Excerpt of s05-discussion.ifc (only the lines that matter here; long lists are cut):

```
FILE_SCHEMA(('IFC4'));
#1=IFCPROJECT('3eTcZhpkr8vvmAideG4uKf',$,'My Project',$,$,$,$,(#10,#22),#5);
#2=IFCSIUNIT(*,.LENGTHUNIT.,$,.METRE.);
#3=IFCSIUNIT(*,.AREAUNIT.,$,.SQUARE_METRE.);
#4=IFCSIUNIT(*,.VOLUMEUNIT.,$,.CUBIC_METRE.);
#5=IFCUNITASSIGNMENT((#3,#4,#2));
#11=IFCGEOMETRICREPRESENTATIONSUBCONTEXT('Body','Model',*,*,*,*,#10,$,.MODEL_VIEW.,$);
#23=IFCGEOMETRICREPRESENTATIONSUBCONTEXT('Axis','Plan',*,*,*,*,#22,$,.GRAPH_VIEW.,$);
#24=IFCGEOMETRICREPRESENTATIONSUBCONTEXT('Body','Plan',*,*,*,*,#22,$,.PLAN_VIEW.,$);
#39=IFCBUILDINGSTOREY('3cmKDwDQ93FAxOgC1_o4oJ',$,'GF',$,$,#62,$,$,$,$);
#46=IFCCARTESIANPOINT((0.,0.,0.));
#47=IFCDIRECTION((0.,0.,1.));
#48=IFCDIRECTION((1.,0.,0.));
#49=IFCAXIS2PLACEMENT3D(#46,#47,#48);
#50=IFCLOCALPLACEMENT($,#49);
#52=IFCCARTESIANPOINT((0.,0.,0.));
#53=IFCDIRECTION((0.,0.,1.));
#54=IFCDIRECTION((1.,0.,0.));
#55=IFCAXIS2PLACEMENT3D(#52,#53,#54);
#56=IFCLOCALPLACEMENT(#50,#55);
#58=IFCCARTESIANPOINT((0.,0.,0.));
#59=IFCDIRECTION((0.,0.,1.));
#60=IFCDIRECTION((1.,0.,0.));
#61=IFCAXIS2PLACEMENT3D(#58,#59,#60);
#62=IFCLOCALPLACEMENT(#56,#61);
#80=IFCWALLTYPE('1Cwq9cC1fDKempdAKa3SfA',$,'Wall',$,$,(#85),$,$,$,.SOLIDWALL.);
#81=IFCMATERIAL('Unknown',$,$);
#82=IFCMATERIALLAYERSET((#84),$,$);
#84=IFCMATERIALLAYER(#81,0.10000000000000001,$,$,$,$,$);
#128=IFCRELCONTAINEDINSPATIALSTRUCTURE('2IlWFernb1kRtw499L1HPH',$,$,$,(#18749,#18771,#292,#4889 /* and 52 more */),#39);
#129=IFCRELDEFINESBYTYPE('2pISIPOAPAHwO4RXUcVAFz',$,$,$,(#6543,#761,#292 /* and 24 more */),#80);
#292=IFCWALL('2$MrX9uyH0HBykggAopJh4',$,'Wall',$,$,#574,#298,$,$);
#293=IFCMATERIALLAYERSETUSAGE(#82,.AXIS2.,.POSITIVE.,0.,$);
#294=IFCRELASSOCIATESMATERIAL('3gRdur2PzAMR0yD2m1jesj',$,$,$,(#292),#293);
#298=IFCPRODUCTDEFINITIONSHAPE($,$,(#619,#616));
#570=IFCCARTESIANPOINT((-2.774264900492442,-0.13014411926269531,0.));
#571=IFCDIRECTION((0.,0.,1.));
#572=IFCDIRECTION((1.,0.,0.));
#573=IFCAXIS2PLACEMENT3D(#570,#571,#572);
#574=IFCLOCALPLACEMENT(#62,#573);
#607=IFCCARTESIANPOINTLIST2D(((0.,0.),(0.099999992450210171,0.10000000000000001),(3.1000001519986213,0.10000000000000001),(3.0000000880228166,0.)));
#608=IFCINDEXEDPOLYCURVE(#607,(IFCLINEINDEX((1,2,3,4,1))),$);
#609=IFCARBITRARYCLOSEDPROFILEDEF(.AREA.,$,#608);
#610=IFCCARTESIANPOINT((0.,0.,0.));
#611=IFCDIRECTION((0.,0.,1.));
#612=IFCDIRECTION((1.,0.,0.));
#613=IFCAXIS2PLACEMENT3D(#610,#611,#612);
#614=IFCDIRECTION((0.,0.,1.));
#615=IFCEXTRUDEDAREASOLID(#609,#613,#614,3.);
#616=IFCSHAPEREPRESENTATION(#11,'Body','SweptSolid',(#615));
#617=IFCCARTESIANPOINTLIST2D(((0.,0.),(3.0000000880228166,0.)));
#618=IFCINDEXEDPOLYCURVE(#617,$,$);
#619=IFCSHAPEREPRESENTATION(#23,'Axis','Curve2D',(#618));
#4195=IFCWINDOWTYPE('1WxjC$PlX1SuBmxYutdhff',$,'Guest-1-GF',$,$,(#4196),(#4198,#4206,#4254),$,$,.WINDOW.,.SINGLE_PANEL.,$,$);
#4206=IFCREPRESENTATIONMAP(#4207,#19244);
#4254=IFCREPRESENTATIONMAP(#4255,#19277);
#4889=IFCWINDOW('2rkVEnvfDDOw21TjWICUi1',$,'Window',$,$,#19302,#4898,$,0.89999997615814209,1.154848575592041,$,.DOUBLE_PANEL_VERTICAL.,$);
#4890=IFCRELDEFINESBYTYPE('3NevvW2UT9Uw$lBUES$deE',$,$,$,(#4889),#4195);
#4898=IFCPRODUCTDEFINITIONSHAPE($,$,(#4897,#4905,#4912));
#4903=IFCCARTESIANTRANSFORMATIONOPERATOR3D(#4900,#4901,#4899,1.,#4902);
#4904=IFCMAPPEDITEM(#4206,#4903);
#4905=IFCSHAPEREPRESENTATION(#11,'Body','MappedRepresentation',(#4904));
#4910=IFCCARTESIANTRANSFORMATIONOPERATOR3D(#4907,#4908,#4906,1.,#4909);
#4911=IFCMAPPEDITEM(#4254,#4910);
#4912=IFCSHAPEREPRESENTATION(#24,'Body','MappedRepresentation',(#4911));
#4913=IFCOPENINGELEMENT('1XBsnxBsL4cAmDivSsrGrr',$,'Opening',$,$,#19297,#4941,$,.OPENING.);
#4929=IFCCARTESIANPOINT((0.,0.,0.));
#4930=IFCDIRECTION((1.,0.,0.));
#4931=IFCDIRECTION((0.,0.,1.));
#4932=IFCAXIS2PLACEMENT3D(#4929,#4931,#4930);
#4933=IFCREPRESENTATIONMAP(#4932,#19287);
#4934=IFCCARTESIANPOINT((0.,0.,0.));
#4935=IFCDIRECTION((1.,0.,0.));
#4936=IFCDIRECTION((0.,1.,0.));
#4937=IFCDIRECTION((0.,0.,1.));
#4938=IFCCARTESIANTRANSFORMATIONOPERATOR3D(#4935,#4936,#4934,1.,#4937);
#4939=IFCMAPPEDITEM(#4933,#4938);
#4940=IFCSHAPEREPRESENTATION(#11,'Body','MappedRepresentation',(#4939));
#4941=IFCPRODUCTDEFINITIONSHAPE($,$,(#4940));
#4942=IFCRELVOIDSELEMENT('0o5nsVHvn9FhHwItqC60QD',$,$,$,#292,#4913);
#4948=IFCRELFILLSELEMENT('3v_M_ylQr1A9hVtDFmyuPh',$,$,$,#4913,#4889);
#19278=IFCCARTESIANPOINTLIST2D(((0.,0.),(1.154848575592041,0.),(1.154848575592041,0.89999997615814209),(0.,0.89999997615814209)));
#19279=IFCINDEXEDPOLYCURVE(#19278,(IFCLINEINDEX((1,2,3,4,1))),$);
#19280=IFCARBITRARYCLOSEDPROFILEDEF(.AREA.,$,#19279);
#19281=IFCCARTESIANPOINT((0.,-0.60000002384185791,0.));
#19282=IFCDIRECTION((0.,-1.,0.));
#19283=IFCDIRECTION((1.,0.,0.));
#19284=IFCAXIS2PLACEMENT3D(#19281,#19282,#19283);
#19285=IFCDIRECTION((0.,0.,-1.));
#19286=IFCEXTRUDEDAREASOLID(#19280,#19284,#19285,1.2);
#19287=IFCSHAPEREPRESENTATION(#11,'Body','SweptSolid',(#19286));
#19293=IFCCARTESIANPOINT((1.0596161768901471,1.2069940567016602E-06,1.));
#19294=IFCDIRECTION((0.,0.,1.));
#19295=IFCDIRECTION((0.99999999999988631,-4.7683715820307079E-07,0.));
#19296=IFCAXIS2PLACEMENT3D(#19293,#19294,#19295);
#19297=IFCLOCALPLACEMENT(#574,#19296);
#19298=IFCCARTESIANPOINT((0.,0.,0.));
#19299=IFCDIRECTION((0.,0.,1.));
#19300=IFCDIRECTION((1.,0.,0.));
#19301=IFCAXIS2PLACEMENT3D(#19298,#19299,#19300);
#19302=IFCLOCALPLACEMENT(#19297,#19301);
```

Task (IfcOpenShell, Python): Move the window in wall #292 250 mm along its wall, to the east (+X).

```python
import ifcopenshell
import ifcopenshell.api.geometry
import ifcopenshell.util.placement
import ifcopenshell.util.unit

model = ifcopenshell.open("s05-discussion.ifc")
unit_scale = ifcopenshell.util.unit.calculate_unit_scale(model)

window = model.by_id(4889)
opening = window.FillsVoids[0].RelatingOpeningElement
wall = opening.VoidsElements[0].RelatingBuildingElement

wall_matrix = ifcopenshell.util.placement.get_local_placement(wall.ObjectPlacement)
shift = wall_matrix[:3, 0] * 0.25 / unit_scale
before = ifcopenshell.util.placement.get_local_placement(window.ObjectPlacement)[:3, 3].copy()

# The window is placed relative to its opening, so it follows when the opening moves.
matrix = ifcopenshell.util.placement.get_local_placement(opening.ObjectPlacement)
matrix[:3, 3] += shift
ifcopenshell.api.geometry.edit_object_placement(
    model, product=opening, matrix=matrix, is_si=False, should_transform_children=True
)

after = ifcopenshell.util.placement.get_local_placement(window.ObjectPlacement)[:3, 3]
print("window moved by", (after - before).round(3) + 0.0)

model.write("s05-discussion_v2.ifc")
```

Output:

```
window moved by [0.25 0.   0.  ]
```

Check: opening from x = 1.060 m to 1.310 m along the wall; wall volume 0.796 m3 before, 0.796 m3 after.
